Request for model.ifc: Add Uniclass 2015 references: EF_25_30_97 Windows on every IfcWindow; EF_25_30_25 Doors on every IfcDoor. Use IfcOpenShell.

First a look at what the model holds.

```python
import ifcopenshell

model = ifcopenshell.open("model.ifc")
print(model.schema)
print("classifications:", [c.Name for c in model.by_type("IfcClassification")])
for ifc_class in ("IfcDoor", "IfcRoof", "IfcStair", "IfcWall", "IfcWindow"):
    print(ifc_class, len(model.by_type(ifc_class)))
```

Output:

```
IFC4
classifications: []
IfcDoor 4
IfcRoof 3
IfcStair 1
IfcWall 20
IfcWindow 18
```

```python
import ifcopenshell
import ifcopenshell.api.classification

model = ifcopenshell.open("model.ifc")

system = ifcopenshell.api.classification.add_classification(model, classification="Uniclass 2015")

codes = {
    "IfcWindow": ("EF_25_30_97", "Windows"),
    "IfcDoor": ("EF_25_30_25", "Doors"),
}
for ifc_class, (code, name) in codes.items():
    products = model.by_type(ifc_class)
    ifcopenshell.api.classification.add_reference(
        model, products=products, classification=system, identification=code, name=name
    )
    print(code, len(products))

model.write("model_updated.ifc")
```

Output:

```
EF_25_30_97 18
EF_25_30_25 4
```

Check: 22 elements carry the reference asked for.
